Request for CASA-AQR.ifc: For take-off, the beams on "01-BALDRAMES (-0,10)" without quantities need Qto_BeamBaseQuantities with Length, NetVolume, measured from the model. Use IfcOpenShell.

First a look at what the model holds.

```python
import ifcopenshell
import ifcopenshell.util.element
import ifcopenshell.util.unit

model = ifcopenshell.open("CASA-AQR.ifc")
print(model.schema)
for unit_type in ("LENGTHUNIT", "AREAUNIT", "VOLUMEUNIT"):
    print(unit_type, ifcopenshell.util.unit.calculate_unit_scale(model, unit_type))
storey = next(s for s in model.by_type("IfcBuildingStorey") if s.Name == "01-BALDRAMES (-0,10)")
beams = [e for e in ifcopenshell.util.element.get_decomposition(storey) if e.is_a("IfcBeam")]
for e in sorted(beams, key=lambda e: e.id()):
    print(e.id(), e.is_a(), e.Name, list(ifcopenshell.util.element.get_psets(e, qtos_only=True)), sep=" | ")
```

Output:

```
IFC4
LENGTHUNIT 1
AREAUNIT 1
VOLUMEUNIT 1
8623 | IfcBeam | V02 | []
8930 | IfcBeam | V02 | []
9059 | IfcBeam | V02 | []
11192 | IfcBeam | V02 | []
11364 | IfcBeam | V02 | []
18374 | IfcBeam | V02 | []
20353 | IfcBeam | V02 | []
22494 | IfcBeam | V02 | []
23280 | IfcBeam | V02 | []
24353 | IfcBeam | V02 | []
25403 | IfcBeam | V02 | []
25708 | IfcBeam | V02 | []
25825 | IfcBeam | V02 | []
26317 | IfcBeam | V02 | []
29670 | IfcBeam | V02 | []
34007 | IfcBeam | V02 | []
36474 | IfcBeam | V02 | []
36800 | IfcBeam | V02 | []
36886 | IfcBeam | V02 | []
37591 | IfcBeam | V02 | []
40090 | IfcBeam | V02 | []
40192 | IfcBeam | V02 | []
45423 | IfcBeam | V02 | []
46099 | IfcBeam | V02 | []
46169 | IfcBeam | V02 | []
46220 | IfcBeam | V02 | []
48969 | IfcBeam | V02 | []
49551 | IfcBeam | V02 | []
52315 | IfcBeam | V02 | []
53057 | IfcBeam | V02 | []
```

```python
import ifcopenshell
import ifcopenshell.api.pset
import ifcopenshell.geom
import ifcopenshell.util.element
import ifcopenshell.util.shape
import ifcopenshell.util.unit

model = ifcopenshell.open("CASA-AQR.ifc")
unit_scale = ifcopenshell.util.unit.calculate_unit_scale(model)
volume_scale = ifcopenshell.util.unit.calculate_unit_scale(model, "VOLUMEUNIT")
settings = ifcopenshell.geom.settings()

storey = next(s for s in model.by_type("IfcBuildingStorey") if s.Name == "01-BALDRAMES (-0,10)")
beams = [e for e in ifcopenshell.util.element.get_decomposition(storey) if e.is_a("IfcBeam")]

for e in sorted(beams, key=lambda e: e.id()):
    if ifcopenshell.util.element.get_psets(e, qtos_only=True, should_inherit=False):
        continue
    # Geometry comes back in metres, in the element's own axes.
    shape = ifcopenshell.geom.create_shape(settings, e)
    values = {
        "Length": ifcopenshell.util.shape.get_max_xyz(shape.geometry) / unit_scale,
        "NetVolume": ifcopenshell.util.shape.get_volume(shape.geometry) / volume_scale,
    }
    qto = ifcopenshell.api.pset.add_qto(model, product=e, name="Qto_BeamBaseQuantities")
    ifcopenshell.api.pset.edit_qto(model, qto=qto, properties=values)
    print(e.id(), {k: round(v, 3) for k, v in values.items()})

model.write("CASA-AQR_v2.ifc")
```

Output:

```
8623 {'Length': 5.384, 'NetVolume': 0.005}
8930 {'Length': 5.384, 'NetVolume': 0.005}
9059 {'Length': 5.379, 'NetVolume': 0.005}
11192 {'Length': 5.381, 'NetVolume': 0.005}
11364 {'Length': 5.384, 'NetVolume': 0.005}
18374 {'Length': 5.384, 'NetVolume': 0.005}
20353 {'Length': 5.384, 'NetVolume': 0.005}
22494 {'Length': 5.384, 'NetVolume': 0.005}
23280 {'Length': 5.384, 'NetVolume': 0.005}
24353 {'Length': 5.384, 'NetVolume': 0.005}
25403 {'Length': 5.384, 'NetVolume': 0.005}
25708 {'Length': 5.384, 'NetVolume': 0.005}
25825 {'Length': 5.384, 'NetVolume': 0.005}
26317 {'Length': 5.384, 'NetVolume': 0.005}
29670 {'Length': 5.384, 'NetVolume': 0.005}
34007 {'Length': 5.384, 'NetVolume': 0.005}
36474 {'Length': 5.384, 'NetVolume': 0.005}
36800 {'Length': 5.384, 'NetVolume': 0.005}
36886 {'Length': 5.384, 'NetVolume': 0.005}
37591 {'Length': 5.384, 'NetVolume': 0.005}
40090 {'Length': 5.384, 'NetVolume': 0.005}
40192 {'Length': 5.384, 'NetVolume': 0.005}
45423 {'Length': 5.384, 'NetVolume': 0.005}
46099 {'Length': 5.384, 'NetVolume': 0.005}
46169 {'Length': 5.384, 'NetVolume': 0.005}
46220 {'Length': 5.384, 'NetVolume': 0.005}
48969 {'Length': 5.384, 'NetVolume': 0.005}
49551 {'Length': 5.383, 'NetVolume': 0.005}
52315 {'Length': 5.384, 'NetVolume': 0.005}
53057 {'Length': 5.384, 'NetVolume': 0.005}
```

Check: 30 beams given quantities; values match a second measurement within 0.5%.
